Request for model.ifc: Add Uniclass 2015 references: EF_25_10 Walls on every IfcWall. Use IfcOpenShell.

First a look at what the model holds.

```python
import ifcopenshell

model = ifcopenshell.open("model.ifc")
print(model.schema)
print("classifications:", [c.Name for c in model.by_type("IfcClassification")])
for ifc_class in ("IfcDoor", "IfcRoof", "IfcStair", "IfcWall", "IfcWindow"):
    print(ifc_class, len(model.by_type(ifc_class)))
```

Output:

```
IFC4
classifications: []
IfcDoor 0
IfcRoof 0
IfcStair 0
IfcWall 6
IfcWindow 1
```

```python
import ifcopenshell
import ifcopenshell.api.classification

model = ifcopenshell.open("model.ifc")

system = ifcopenshell.api.classification.add_classification(model, classification="Uniclass 2015")

codes = {
    "IfcWall": ("EF_25_10", "Walls"),
}
for ifc_class, (code, name) in codes.items():
    products = model.by_type(ifc_class)
    ifcopenshell.api.classification.add_reference(
        model, products=products, classification=system, identification=code, name=name
    )
    print(code, len(products))

model.write("model_v2.ifc")
```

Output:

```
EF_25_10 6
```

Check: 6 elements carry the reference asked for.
